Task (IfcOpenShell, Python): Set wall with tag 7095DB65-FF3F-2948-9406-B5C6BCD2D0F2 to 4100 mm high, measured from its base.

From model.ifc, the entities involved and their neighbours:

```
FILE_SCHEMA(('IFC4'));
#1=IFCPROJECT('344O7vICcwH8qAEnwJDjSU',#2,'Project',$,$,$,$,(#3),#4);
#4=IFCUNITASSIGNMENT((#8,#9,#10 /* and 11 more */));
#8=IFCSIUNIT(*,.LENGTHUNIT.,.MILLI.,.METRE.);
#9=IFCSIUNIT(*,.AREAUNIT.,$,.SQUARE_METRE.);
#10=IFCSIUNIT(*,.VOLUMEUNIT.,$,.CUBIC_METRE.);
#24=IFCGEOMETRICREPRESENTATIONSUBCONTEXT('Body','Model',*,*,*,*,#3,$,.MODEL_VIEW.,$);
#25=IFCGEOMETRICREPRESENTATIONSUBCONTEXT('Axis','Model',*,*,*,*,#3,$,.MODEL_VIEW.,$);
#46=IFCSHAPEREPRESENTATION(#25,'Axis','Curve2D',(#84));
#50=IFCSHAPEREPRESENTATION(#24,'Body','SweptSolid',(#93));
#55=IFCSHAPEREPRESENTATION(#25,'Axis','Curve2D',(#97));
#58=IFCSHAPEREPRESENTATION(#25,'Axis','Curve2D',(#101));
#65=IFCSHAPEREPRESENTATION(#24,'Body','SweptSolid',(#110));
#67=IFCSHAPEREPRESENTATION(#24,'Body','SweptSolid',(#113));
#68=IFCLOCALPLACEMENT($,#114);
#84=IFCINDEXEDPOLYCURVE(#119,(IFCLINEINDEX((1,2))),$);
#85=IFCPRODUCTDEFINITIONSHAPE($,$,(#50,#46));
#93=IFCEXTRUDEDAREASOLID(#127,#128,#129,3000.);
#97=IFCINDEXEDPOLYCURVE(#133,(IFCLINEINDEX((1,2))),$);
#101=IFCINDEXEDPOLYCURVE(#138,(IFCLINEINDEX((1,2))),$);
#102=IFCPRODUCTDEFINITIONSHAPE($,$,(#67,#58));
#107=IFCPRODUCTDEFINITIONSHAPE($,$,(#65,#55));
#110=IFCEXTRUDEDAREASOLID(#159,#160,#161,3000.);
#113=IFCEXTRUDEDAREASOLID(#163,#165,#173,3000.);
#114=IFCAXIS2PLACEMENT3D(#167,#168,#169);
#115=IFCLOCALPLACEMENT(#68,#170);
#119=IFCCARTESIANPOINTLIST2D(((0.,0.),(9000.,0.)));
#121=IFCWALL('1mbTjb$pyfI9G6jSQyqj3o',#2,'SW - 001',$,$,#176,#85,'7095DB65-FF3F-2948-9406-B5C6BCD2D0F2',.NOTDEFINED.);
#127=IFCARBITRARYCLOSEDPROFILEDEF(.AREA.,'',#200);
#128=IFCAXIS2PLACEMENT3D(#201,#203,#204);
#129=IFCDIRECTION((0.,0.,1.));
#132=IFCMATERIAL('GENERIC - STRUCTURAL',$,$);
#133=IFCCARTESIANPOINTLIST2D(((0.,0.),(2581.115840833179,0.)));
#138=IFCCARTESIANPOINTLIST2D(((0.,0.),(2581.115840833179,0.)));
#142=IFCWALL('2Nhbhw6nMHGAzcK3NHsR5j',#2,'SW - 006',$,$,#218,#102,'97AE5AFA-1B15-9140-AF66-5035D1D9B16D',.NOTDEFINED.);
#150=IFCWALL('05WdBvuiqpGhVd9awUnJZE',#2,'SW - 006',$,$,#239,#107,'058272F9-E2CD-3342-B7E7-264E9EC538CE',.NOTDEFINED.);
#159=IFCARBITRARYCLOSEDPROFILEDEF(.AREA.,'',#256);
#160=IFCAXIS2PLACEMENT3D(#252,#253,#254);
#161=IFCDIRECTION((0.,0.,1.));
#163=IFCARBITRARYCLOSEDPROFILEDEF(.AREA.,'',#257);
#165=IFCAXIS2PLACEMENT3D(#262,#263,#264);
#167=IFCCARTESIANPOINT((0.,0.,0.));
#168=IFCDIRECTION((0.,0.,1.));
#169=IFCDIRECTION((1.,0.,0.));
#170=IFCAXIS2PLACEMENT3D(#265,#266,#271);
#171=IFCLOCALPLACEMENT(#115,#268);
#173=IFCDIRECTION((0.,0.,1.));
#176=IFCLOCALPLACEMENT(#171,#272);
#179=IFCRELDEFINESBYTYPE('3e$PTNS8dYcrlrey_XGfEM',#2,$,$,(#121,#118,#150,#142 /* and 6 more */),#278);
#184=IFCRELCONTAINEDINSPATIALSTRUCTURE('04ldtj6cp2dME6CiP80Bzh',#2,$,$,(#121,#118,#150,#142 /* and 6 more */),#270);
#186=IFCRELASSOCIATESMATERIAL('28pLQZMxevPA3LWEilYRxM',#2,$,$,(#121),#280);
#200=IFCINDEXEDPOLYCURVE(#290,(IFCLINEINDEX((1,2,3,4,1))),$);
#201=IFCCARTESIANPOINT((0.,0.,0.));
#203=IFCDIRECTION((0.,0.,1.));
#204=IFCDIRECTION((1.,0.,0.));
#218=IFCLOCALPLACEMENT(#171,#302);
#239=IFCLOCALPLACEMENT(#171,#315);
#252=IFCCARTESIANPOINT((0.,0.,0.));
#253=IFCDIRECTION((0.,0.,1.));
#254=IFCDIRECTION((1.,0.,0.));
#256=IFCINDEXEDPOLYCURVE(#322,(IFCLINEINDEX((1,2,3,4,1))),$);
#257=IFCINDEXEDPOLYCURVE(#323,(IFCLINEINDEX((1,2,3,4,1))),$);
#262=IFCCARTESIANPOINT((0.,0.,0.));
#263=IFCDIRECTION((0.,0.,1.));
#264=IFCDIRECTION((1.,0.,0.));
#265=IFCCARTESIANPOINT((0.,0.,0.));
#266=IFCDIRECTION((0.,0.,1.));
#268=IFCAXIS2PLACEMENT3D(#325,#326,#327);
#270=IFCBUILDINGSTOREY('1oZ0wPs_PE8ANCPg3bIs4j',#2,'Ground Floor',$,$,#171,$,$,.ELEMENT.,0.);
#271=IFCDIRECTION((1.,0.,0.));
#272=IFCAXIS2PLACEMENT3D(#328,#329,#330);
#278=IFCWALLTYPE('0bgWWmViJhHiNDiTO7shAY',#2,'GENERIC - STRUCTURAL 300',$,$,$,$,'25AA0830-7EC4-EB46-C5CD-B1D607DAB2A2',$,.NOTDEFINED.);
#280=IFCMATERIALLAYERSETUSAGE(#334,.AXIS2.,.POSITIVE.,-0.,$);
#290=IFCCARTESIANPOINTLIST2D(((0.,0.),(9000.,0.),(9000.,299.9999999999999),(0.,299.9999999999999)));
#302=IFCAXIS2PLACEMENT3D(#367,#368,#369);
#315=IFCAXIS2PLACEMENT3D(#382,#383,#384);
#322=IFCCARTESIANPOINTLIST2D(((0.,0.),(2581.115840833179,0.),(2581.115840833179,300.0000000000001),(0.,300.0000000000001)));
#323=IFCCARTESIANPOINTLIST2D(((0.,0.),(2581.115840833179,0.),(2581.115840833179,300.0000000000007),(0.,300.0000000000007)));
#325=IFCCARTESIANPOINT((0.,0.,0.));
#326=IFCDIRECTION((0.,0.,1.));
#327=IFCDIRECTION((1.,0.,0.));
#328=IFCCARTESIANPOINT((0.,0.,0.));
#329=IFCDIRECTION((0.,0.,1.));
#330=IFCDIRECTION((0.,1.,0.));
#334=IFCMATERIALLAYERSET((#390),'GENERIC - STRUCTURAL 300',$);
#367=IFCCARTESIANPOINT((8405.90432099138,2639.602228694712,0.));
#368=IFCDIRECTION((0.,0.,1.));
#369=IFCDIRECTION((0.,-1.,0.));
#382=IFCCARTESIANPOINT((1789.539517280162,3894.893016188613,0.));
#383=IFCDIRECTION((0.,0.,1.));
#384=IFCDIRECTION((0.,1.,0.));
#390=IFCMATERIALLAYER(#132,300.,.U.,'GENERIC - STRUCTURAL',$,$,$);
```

```python
import ifcopenshell
import ifcopenshell.geom
import ifcopenshell.util.representation
import ifcopenshell.util.shape
import ifcopenshell.util.unit

model = ifcopenshell.open("model.ifc")
unit_scale = ifcopenshell.util.unit.calculate_unit_scale(model)
settings = ifcopenshell.geom.settings()


def volume(element):
    """Net volume in cubic metres, openings subtracted."""
    shape = ifcopenshell.geom.create_shape(settings, element)
    return ifcopenshell.util.shape.get_volume(shape.geometry)


wall = model.by_guid("1mbTjb$pyfI9G6jSQyqj3o")
before = volume(wall)

body = ifcopenshell.util.representation.get_representation(wall, "Model", "Body")
solid = body.Items[0]
old_height = solid.Depth
solid.Depth = 4.1 / unit_scale
after = volume(wall)

print(f"height {old_height:g} -> {solid.Depth:g}, volume {before:.3f} -> {after:.3f} m3")

model.write("model_updated.ifc")
```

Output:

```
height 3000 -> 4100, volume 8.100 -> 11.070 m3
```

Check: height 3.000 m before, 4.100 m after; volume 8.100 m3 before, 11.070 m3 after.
